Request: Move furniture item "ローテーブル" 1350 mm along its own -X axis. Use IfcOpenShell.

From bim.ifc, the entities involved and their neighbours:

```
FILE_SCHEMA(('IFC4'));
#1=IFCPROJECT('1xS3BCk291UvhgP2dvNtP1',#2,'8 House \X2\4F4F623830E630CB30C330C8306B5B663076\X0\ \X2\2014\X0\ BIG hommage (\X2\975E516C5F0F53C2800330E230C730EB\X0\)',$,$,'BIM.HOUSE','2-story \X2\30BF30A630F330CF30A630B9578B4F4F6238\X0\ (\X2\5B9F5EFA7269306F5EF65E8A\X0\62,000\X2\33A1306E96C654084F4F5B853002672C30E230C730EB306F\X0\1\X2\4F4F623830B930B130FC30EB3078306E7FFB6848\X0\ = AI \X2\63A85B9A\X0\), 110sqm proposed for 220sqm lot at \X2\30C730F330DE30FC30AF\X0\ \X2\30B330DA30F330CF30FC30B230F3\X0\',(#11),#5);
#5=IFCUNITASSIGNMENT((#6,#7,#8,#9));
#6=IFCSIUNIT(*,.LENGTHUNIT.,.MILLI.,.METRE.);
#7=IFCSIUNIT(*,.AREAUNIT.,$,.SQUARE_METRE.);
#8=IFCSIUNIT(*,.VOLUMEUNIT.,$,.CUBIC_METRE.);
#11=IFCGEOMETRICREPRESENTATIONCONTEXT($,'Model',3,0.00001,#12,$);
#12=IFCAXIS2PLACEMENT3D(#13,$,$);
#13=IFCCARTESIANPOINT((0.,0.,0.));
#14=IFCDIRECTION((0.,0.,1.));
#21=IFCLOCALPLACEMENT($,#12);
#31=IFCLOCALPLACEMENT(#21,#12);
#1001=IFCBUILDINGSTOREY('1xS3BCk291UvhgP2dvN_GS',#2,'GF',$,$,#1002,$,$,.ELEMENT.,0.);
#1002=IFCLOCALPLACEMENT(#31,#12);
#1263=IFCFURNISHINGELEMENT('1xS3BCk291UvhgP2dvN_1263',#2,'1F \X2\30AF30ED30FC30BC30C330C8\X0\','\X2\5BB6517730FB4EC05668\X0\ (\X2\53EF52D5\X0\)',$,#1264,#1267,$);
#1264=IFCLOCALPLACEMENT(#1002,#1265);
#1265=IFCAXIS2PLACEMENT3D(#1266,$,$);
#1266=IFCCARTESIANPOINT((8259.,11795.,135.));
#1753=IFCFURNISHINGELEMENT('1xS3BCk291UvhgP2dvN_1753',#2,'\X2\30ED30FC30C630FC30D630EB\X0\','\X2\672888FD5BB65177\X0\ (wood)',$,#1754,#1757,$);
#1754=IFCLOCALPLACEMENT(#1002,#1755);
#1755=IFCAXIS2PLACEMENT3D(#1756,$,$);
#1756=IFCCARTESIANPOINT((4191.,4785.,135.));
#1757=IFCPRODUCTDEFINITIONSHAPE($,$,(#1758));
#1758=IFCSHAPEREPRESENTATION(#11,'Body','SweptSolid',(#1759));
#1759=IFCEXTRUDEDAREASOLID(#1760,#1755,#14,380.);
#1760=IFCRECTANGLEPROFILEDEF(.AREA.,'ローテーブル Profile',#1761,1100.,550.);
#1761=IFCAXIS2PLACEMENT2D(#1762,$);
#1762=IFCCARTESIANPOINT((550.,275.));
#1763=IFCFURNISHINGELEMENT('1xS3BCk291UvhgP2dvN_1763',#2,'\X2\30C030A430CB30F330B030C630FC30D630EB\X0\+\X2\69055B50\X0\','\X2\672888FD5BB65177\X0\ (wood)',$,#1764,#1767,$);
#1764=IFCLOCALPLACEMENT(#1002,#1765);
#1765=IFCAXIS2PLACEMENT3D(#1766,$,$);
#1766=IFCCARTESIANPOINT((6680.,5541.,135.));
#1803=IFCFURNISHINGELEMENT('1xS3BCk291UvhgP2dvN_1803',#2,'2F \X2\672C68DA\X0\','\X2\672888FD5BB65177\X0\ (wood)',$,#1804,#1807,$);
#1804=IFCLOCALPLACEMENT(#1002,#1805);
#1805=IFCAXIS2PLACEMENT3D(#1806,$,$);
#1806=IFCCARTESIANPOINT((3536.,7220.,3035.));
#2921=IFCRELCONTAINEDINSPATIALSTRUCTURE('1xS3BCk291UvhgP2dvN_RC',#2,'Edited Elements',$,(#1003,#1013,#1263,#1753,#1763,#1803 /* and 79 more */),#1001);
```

```python
import ifcopenshell
import ifcopenshell.api.geometry
import ifcopenshell.util.placement
import ifcopenshell.util.unit

model = ifcopenshell.open("bim.ifc")
unit_scale = ifcopenshell.util.unit.calculate_unit_scale(model)

item = model.by_guid("1xS3BCk291UvhgP2dvN_1753")
matrix = ifcopenshell.util.placement.get_local_placement(item.ObjectPlacement)
matrix[:3, 3] -= matrix[:3, 0] * 1.35 / unit_scale
ifcopenshell.api.geometry.edit_object_placement(model, product=item, matrix=matrix, is_si=False)

print(ifcopenshell.util.placement.get_local_placement(item.ObjectPlacement).round(3) + 0.0)

model.write("bim_updated.ifc")
```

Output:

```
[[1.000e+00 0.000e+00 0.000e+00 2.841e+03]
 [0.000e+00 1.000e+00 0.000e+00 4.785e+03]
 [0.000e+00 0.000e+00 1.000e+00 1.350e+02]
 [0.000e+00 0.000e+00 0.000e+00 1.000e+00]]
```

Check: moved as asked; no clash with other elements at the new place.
